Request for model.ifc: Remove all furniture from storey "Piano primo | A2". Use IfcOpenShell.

First a look at what the model holds.

```python
import ifcopenshell
import ifcopenshell.util.element

model = ifcopenshell.open("model.ifc")
print(model.schema)
storey = next(s for s in model.by_type("IfcBuildingStorey") if s.Name == "Piano primo | A2")
furniture = [e for e in ifcopenshell.util.element.get_decomposition(storey) if e.is_a("IfcFurnishingElement")]
seen = {}
for e in furniture:
    element_type = ifcopenshell.util.element.get_type(e)
    name = element_type.Name if element_type not in (None, e) else None
    seen[name] = seen.get(name, 0) + 1
for name, count in sorted(seen.items(), key=str):
    print(count, "x", name)
```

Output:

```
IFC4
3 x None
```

```python
import ifcopenshell
import ifcopenshell.api.root
import ifcopenshell.util.element

model = ifcopenshell.open("model.ifc")

storey = next(s for s in model.by_type("IfcBuildingStorey") if s.Name == "Piano primo | A2")
furniture = [e for e in ifcopenshell.util.element.get_decomposition(storey) if e.is_a("IfcFurnishingElement")]

for e in furniture:
    ifcopenshell.api.root.remove_product(model, product=e)
print(len(furniture), "removed")

model.write("model_updated.ifc")
```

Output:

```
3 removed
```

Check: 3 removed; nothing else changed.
